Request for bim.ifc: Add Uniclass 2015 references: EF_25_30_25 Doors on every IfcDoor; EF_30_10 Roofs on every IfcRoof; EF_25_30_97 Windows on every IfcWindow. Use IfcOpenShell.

First a look at what the model holds.

```python
import ifcopenshell

model = ifcopenshell.open("bim.ifc")
print(model.schema)
print("classifications:", [c.Name for c in model.by_type("IfcClassification")])
for ifc_class in ("IfcDoor", "IfcRoof", "IfcStair", "IfcWall", "IfcWindow"):
    print(ifc_class, len(model.by_type(ifc_class)))
```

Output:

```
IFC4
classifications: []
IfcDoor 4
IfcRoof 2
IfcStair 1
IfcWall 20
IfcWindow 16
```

```python
import ifcopenshell
import ifcopenshell.api.classification

model = ifcopenshell.open("bim.ifc")

system = ifcopenshell.api.classification.add_classification(model, classification="Uniclass 2015")

codes = {
    "IfcDoor": ("EF_25_30_25", "Doors"),
    "IfcRoof": ("EF_30_10", "Roofs"),
    "IfcWindow": ("EF_25_30_97", "Windows"),
}
for ifc_class, (code, name) in codes.items():
    products = model.by_type(ifc_class)
    ifcopenshell.api.classification.add_reference(
        model, products=products, classification=system, identification=code, name=name
    )
    print(code, len(products))

model.write("bim-out.ifc")
```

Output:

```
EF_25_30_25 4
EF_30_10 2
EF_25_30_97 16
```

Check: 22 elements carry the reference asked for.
